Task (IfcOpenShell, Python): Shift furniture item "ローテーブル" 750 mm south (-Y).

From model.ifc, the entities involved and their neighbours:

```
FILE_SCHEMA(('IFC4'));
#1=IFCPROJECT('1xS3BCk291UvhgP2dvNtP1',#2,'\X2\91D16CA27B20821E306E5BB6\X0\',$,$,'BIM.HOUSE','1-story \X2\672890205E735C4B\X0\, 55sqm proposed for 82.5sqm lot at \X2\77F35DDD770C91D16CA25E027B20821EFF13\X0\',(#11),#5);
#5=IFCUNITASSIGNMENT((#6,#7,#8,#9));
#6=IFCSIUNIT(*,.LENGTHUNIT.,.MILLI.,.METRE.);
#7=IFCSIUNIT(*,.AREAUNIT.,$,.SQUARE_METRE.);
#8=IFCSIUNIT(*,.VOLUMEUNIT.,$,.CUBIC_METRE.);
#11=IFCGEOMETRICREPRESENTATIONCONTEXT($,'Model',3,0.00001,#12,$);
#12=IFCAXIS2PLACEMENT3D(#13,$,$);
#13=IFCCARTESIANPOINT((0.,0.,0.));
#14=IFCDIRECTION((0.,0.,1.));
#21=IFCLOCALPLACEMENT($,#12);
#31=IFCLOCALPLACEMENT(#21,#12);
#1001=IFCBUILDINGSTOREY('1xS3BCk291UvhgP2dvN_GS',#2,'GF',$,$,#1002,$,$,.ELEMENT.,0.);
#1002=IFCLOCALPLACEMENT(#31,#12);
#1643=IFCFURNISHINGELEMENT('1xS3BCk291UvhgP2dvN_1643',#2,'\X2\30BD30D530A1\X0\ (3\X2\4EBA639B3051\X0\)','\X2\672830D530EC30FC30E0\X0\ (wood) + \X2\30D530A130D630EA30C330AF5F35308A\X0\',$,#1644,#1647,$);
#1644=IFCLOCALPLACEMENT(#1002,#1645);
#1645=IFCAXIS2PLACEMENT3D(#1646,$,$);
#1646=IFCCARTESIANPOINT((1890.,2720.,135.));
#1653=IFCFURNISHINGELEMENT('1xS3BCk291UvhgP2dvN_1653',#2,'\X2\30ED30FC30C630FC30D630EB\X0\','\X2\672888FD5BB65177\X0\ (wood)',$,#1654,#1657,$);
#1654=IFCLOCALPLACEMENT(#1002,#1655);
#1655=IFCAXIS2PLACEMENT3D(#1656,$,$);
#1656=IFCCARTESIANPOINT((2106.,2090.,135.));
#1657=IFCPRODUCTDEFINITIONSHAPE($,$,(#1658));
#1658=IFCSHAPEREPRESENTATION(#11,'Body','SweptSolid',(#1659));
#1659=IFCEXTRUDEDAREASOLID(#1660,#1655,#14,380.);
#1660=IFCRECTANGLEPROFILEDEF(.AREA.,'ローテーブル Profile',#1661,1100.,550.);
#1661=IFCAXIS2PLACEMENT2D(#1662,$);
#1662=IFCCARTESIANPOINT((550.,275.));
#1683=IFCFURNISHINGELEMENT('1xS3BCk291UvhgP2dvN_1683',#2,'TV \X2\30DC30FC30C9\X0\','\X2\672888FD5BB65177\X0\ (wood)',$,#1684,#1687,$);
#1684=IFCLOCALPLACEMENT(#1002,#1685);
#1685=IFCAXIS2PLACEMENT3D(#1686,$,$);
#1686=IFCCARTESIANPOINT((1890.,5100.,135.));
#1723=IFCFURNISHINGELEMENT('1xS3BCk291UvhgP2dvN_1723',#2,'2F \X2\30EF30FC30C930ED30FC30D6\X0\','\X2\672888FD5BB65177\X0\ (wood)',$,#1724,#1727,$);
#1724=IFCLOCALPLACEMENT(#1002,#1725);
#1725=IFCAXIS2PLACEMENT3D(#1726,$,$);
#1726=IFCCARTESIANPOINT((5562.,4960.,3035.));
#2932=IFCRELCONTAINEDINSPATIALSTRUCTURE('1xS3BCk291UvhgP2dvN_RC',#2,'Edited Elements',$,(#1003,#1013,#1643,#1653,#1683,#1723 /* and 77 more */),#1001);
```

```python
import ifcopenshell
import ifcopenshell.api.geometry
import ifcopenshell.util.placement
import ifcopenshell.util.unit

model = ifcopenshell.open("model.ifc")
unit_scale = ifcopenshell.util.unit.calculate_unit_scale(model)

item = model.by_guid("1xS3BCk291UvhgP2dvN_1653")
matrix = ifcopenshell.util.placement.get_local_placement(item.ObjectPlacement)
matrix[1, 3] -= 0.75 / unit_scale
ifcopenshell.api.geometry.edit_object_placement(model, product=item, matrix=matrix, is_si=False)

print(ifcopenshell.util.placement.get_local_placement(item.ObjectPlacement).round(3) + 0.0)

model.write("model_v2.ifc")
```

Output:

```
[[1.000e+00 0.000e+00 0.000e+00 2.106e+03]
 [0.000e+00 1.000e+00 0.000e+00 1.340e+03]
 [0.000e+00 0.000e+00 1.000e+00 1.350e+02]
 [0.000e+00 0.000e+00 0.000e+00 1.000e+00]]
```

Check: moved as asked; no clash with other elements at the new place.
